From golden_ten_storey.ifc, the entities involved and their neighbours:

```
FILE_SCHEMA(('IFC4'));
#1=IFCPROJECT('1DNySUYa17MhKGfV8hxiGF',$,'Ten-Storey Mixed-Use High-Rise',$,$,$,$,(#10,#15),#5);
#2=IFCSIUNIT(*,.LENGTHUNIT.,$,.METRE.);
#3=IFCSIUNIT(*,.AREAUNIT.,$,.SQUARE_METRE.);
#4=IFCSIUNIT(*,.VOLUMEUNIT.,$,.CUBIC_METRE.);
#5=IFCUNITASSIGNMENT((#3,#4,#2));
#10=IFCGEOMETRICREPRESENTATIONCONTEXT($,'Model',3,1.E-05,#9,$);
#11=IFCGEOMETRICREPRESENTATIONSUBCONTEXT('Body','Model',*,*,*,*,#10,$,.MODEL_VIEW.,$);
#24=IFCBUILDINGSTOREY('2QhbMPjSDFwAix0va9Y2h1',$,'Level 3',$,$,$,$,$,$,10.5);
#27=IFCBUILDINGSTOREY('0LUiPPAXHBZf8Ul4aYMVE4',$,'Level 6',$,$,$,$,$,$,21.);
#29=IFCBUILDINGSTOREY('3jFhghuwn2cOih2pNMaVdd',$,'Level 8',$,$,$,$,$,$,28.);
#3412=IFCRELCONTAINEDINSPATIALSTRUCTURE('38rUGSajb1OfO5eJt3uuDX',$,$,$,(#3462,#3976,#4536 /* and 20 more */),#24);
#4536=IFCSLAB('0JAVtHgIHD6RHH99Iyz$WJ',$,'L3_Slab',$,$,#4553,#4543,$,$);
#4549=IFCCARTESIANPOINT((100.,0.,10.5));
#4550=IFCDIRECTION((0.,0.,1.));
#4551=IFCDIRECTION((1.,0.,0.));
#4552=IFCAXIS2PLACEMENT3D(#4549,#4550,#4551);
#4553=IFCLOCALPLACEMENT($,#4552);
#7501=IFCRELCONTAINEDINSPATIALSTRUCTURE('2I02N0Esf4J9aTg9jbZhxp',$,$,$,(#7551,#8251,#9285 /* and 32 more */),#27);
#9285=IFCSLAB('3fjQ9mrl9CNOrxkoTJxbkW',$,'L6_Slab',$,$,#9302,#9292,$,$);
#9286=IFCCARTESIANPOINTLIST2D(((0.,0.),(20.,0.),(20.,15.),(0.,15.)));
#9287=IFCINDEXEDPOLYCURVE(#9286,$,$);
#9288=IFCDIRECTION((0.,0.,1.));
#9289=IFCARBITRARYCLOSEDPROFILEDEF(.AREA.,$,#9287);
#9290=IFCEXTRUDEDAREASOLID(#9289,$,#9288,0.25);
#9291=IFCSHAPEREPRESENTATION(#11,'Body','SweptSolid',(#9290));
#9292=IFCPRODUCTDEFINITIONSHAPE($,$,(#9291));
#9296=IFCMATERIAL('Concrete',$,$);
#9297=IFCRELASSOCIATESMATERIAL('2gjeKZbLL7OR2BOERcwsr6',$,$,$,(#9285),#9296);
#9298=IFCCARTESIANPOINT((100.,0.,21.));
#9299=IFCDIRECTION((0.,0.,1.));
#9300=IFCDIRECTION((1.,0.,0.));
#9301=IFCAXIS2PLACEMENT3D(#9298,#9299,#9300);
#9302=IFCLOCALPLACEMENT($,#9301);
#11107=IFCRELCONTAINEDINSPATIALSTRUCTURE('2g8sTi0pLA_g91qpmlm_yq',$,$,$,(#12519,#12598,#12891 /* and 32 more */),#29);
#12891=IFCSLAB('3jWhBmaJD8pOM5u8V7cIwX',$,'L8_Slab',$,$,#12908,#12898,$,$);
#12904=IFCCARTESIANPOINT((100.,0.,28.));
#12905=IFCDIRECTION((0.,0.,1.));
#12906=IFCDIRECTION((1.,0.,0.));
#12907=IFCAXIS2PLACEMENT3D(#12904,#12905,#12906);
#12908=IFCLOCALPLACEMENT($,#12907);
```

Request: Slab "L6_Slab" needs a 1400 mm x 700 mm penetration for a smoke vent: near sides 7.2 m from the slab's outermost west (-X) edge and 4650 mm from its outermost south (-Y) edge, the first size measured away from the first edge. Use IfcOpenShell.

```python
import numpy as np
import ifcopenshell
import ifcopenshell.api.feature
import ifcopenshell.api.geometry
import ifcopenshell.api.root
import ifcopenshell.geom
import ifcopenshell.util.placement
import ifcopenshell.util.representation
import ifcopenshell.util.shape
import ifcopenshell.util.unit

model = ifcopenshell.open("golden_ten_storey.ifc")
unit_scale = ifcopenshell.util.unit.calculate_unit_scale(model)
settings = ifcopenshell.geom.settings()


def volume(element):
    """Net volume in cubic metres, openings subtracted."""
    shape = ifcopenshell.geom.create_shape(settings, element)
    return ifcopenshell.util.shape.get_volume(shape.geometry)


slab = model.by_id(9285)
before = volume(slab)

# Extent in the slab's own axes, in metres. The edges named are its -X and -Y sides.
slab_shape = ifcopenshell.geom.create_shape(settings, slab)
vertices = ifcopenshell.util.shape.get_vertices(slab_shape.geometry)
x_min, y_min, bottom = vertices.min(axis=0)
top = vertices[:, 2].max()

opening = ifcopenshell.api.root.create_entity(model, ifc_class="IfcOpeningElement", name="Smoke vent opening", predefined_type="OPENING")
context = ifcopenshell.util.representation.get_context(model, "Model", "Body", "MODEL_VIEW")
width, depth = 1.4, 0.7
outline = [(0.0, 0.0), (width, 0.0), (width, depth), (0.0, depth), (0.0, 0.0)]
# Overshoot both faces by 50 mm so the cut is clean.
shape = ifcopenshell.api.geometry.add_slab_representation(
    model, context=context, depth=top - bottom + 0.1, polyline=outline
)
ifcopenshell.api.geometry.assign_representation(model, product=opening, representation=shape)

matrix = ifcopenshell.util.placement.get_local_placement(slab.ObjectPlacement)
matrix[:, 3] = matrix @ np.append(np.array([x_min + 7.2, y_min + 4.65, bottom - 0.05]) / unit_scale, 1.0)
ifcopenshell.api.geometry.edit_object_placement(model, product=opening, matrix=matrix, is_si=False)
ifcopenshell.api.feature.add_feature(model, feature=opening, element=slab)

after = volume(slab)

print(f"slab volume {before:.3f} -> {after:.3f} m3")

model.write("golden_ten_storey_updated.ifc")
```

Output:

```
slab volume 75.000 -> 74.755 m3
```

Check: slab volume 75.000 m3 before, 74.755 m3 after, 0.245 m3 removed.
